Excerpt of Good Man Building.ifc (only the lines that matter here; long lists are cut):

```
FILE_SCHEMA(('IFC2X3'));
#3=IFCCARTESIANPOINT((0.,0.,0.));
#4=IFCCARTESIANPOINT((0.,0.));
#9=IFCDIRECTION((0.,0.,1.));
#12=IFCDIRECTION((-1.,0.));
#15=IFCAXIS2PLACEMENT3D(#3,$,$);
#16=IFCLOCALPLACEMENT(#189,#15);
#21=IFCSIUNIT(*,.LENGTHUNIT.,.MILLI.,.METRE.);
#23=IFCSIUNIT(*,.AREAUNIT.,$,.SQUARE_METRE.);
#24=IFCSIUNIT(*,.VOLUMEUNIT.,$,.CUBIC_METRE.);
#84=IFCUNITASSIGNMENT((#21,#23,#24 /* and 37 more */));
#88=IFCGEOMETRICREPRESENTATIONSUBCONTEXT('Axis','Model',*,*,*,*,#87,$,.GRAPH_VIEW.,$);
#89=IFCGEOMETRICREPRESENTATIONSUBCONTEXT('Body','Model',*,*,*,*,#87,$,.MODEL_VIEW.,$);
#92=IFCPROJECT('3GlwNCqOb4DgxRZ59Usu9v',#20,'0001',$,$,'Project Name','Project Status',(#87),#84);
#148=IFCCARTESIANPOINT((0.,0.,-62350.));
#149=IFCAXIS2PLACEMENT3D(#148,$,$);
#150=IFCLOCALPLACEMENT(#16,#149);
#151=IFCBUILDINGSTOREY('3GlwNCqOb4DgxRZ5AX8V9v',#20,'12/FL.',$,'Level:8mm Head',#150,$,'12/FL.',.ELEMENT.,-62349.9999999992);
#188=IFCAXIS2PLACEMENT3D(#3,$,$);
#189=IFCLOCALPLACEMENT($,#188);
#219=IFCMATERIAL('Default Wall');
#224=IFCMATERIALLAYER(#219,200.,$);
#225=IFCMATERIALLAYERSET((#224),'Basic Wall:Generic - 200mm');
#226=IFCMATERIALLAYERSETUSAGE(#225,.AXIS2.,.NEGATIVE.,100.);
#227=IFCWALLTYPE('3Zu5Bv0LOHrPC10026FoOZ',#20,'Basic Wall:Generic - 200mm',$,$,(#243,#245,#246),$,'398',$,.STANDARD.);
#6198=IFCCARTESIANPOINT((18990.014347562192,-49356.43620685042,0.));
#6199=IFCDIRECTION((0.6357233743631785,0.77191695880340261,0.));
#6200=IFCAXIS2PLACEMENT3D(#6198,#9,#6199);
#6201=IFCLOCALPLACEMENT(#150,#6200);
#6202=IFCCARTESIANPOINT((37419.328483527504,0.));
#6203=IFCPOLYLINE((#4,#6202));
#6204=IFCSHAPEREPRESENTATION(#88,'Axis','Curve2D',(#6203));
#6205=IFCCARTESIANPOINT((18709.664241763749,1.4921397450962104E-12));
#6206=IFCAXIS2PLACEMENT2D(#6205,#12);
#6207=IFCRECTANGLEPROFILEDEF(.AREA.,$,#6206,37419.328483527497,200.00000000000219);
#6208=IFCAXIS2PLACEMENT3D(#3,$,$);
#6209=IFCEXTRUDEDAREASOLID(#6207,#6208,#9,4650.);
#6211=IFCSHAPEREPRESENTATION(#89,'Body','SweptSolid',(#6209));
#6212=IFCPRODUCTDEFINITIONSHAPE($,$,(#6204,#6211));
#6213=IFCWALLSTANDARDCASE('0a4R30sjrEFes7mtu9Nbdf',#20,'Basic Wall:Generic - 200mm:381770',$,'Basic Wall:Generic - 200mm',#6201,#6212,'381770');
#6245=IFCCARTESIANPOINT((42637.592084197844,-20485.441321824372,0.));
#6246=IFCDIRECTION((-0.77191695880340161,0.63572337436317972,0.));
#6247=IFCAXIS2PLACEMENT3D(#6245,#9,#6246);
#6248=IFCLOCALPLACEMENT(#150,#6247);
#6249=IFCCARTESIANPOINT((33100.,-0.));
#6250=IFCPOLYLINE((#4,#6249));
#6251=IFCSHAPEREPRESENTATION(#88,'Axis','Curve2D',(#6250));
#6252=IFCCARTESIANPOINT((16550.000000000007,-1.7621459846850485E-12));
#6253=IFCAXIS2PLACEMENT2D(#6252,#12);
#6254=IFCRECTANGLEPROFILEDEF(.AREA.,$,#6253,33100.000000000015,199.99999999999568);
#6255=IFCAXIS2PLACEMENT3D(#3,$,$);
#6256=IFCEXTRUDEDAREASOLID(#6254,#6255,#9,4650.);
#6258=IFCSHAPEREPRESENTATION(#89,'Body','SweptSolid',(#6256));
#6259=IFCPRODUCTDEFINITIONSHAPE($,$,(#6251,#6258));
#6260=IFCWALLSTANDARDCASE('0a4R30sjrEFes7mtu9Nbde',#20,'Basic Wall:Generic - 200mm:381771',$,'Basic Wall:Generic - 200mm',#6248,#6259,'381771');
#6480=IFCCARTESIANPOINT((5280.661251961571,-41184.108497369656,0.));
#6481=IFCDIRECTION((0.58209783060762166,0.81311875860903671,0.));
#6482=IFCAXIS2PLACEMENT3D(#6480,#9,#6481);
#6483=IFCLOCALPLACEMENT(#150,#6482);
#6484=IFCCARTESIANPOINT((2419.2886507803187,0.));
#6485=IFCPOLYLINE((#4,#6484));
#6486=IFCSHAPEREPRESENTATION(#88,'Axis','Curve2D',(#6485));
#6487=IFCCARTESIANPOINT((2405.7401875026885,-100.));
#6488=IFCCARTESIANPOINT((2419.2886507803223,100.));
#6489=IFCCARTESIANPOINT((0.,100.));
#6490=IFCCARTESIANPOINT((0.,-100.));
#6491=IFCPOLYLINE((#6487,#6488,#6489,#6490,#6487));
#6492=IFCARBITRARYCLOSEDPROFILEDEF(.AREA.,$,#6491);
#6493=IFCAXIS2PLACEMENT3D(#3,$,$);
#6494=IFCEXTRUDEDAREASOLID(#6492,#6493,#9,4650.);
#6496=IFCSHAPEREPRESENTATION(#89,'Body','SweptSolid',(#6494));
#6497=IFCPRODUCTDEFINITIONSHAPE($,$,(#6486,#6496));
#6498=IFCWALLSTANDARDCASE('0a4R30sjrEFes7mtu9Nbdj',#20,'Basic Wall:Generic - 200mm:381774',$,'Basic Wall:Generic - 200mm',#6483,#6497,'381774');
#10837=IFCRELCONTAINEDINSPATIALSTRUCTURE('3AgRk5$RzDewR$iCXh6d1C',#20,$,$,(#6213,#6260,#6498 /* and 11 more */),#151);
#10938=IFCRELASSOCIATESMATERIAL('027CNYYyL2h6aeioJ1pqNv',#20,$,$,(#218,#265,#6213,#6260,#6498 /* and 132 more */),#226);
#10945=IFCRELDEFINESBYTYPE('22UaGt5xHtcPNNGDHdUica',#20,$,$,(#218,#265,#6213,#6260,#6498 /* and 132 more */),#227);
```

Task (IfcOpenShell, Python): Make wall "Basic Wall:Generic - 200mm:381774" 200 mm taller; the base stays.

```python
import ifcopenshell
import ifcopenshell.geom
import ifcopenshell.util.representation
import ifcopenshell.util.shape

model = ifcopenshell.open("Good Man Building.ifc")
settings = ifcopenshell.geom.settings()


def volume(element):
    """Net volume in cubic metres, openings subtracted."""
    shape = ifcopenshell.geom.create_shape(settings, element)
    return ifcopenshell.util.shape.get_volume(shape.geometry)


wall = model.by_guid("0a4R30sjrEFes7mtu9Nbdj")
before = volume(wall)

body = ifcopenshell.util.representation.get_representation(wall, "Model", "Body")
solid = body.Items[0]
old_height = solid.Depth
solid.Depth += 200.0
after = volume(wall)

print(f"height {old_height:g} -> {solid.Depth:g}, volume {before:.3f} -> {after:.3f} m3")

model.write("Good Man Building_edited.ifc")
```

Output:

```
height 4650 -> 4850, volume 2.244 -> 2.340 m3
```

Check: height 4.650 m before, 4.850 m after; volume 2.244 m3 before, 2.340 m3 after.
